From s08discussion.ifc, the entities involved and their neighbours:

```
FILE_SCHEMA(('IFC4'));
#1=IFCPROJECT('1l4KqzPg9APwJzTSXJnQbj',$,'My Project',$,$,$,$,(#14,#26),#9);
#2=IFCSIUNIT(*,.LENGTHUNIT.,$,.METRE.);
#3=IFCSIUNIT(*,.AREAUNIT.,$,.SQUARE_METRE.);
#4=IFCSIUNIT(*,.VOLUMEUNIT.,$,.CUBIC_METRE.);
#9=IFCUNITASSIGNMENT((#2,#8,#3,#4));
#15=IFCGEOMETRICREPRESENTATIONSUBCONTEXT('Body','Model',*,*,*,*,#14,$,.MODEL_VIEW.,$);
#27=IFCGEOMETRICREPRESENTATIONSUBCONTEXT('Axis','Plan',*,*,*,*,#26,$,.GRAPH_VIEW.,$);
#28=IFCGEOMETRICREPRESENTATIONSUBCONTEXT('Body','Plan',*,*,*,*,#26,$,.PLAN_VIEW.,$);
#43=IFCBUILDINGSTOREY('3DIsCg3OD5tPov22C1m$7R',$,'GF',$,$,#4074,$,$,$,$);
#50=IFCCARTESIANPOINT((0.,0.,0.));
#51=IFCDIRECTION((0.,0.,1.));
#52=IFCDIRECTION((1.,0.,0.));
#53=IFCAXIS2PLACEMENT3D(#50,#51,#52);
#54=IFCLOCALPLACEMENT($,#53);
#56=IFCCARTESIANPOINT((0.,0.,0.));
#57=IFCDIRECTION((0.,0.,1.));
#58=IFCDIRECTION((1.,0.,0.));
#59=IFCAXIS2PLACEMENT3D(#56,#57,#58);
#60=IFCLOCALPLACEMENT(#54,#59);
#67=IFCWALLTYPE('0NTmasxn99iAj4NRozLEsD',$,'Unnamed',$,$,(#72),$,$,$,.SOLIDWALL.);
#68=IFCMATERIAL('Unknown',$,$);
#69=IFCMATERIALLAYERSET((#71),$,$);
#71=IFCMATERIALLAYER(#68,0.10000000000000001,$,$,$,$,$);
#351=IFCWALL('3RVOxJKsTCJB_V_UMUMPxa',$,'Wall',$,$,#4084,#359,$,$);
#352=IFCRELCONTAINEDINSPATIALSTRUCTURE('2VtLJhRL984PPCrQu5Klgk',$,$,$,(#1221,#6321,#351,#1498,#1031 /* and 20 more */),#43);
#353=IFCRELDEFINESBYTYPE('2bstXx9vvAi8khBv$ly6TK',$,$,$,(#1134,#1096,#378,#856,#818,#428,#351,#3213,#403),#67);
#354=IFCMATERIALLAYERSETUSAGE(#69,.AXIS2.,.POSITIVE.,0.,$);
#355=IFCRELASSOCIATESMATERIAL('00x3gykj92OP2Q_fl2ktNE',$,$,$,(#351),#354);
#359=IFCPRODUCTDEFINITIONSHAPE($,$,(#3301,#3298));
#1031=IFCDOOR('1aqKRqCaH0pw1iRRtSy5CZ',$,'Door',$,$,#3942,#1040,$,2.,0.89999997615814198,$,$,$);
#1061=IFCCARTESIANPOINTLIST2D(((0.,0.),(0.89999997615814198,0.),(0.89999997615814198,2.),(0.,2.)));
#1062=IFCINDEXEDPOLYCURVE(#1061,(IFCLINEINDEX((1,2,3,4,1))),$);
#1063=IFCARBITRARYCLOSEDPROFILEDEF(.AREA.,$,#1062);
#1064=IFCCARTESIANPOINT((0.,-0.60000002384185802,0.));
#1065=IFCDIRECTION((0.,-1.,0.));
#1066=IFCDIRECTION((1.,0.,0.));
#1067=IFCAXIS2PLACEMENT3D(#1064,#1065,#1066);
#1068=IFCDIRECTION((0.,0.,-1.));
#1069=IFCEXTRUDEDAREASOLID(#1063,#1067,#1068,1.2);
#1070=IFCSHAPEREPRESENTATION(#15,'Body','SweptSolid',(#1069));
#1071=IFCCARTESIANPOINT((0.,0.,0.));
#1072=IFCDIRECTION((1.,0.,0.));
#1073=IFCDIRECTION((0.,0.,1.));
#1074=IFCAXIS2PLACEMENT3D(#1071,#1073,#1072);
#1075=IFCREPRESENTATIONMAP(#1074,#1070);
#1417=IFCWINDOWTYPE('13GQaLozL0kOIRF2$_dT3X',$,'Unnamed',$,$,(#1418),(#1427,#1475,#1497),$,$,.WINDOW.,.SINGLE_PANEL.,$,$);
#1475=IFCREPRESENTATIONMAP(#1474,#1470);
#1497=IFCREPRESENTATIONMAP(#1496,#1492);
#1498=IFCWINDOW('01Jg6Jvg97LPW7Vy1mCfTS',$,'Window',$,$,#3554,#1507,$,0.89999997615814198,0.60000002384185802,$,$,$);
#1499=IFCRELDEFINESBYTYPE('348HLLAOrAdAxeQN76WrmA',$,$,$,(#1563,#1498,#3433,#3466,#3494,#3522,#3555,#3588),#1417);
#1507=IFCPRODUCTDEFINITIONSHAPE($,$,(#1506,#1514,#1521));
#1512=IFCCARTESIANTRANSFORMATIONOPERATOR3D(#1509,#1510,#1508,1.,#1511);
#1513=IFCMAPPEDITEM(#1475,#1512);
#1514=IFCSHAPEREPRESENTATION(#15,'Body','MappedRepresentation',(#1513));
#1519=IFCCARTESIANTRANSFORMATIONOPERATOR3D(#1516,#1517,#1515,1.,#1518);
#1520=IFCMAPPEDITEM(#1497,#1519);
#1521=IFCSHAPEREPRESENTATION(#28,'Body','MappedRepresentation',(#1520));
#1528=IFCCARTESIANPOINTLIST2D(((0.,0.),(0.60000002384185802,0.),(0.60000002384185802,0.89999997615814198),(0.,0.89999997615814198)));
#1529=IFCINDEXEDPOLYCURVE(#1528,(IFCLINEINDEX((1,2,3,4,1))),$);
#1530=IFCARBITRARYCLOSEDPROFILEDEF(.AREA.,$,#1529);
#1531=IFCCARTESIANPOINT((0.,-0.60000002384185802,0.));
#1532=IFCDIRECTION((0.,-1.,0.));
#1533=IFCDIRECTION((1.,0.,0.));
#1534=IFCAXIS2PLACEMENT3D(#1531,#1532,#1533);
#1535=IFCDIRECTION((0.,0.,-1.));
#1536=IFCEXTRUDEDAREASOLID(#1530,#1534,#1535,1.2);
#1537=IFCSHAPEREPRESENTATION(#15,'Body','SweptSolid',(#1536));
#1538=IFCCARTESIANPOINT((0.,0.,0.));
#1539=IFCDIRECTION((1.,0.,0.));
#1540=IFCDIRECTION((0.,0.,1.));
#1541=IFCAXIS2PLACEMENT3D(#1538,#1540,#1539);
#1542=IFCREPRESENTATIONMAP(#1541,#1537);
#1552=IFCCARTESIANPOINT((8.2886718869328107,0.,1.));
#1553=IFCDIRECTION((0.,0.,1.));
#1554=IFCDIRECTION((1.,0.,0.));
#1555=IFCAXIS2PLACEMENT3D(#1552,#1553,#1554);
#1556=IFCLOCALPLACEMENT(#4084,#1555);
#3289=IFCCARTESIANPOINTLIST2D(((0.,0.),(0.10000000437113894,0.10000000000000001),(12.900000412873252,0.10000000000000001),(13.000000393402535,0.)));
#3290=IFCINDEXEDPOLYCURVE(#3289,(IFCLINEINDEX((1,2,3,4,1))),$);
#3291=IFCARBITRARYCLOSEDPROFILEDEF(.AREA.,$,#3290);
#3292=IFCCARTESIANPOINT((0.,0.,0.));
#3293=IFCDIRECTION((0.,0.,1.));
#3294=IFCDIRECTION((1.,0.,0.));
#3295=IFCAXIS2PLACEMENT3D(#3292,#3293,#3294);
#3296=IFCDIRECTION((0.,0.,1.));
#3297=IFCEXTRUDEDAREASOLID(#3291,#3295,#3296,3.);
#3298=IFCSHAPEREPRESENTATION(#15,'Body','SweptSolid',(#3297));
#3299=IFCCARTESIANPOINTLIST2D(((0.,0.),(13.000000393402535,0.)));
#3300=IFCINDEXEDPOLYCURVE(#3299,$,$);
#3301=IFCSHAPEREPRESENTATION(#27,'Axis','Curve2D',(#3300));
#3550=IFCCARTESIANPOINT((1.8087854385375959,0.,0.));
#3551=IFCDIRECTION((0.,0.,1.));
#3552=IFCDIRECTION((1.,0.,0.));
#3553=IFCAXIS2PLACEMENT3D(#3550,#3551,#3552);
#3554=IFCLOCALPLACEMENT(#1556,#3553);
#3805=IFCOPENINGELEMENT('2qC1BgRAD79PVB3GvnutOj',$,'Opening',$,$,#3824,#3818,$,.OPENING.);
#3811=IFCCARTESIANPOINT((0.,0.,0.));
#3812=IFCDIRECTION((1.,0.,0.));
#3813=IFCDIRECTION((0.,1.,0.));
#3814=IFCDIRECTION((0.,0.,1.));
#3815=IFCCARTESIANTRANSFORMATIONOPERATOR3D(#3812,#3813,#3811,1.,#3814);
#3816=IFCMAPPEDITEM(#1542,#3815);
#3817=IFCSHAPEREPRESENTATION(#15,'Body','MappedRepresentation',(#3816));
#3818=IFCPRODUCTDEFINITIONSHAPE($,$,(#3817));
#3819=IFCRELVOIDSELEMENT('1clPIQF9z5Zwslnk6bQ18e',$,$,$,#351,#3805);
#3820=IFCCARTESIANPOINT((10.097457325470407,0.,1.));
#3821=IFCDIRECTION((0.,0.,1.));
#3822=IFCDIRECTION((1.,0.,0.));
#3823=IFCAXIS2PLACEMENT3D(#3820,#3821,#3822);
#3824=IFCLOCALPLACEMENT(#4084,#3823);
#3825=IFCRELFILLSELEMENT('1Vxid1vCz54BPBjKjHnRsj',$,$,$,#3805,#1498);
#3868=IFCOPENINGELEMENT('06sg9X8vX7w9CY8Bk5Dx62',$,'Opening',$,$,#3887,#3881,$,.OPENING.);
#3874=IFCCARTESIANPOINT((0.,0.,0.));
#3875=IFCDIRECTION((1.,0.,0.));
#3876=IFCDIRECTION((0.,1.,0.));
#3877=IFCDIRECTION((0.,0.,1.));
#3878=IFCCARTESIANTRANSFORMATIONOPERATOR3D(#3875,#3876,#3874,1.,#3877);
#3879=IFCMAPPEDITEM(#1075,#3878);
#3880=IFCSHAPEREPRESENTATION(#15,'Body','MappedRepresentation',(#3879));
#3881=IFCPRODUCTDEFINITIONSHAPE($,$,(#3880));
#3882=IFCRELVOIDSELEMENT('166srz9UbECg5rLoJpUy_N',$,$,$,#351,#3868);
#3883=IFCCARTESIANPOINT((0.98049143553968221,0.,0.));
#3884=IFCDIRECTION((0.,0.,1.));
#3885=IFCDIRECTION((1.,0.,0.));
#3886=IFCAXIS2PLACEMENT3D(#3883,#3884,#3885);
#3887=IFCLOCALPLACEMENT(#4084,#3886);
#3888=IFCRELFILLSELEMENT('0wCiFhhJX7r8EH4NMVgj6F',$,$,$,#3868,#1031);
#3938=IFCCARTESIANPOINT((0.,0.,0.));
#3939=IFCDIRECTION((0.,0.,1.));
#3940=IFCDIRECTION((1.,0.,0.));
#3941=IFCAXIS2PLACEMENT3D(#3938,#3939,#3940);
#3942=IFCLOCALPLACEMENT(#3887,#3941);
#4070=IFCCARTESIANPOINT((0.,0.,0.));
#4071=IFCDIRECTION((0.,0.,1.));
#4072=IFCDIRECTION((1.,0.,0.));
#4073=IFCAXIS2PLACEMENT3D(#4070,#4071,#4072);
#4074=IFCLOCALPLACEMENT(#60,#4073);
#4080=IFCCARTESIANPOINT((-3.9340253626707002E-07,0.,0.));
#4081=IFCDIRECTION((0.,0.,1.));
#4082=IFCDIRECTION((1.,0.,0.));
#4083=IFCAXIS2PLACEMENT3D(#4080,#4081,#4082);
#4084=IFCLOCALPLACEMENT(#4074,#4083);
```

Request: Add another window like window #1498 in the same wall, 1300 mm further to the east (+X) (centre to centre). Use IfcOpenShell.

```python
import ifcopenshell
import ifcopenshell.api.feature
import ifcopenshell.api.geometry
import ifcopenshell.api.root
import ifcopenshell.geom
import ifcopenshell.util.element
import ifcopenshell.util.placement
import ifcopenshell.util.shape
import ifcopenshell.util.unit

model = ifcopenshell.open("s08discussion.ifc")
unit_scale = ifcopenshell.util.unit.calculate_unit_scale(model)
settings = ifcopenshell.geom.settings()


def volume(element):
    """Net volume in cubic metres, openings subtracted."""
    shape = ifcopenshell.geom.create_shape(settings, element)
    return ifcopenshell.util.shape.get_volume(shape.geometry)


window = model.by_id(1498)
opening = window.FillsVoids[0].RelatingOpeningElement
wall = opening.VoidsElements[0].RelatingBuildingElement
before = volume(wall)
shift = ifcopenshell.util.placement.get_local_placement(wall.ObjectPlacement)[:3, 0] * 1.3 / unit_scale

# copy_class copies the void relationship, type, container and properties, but no geometry.
new_opening = ifcopenshell.api.root.copy_class(model, product=opening)
new_opening.Representation = ifcopenshell.util.element.copy_deep(
    model, opening.Representation, exclude=["IfcGeometricRepresentationContext", "IfcRepresentationMap"]
)
new_window = ifcopenshell.api.root.copy_class(model, product=window)
new_window.Representation = ifcopenshell.util.element.copy_deep(
    model, window.Representation, exclude=["IfcGeometricRepresentationContext", "IfcRepresentationMap"]
)
ifcopenshell.api.feature.add_filling(model, opening=new_opening, element=new_window)

for old, new in ((opening, new_opening), (window, new_window)):
    matrix = ifcopenshell.util.placement.get_local_placement(old.ObjectPlacement)
    matrix[:3, 3] += shift
    ifcopenshell.api.geometry.edit_object_placement(model, product=new, matrix=matrix, is_si=False)

after = volume(wall)

print(f"wall volume {before:.3f} -> {after:.3f} m3")

model.write("s08discussion_rev.ifc")
```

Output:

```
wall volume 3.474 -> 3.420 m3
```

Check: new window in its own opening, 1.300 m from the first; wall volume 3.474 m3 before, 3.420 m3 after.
